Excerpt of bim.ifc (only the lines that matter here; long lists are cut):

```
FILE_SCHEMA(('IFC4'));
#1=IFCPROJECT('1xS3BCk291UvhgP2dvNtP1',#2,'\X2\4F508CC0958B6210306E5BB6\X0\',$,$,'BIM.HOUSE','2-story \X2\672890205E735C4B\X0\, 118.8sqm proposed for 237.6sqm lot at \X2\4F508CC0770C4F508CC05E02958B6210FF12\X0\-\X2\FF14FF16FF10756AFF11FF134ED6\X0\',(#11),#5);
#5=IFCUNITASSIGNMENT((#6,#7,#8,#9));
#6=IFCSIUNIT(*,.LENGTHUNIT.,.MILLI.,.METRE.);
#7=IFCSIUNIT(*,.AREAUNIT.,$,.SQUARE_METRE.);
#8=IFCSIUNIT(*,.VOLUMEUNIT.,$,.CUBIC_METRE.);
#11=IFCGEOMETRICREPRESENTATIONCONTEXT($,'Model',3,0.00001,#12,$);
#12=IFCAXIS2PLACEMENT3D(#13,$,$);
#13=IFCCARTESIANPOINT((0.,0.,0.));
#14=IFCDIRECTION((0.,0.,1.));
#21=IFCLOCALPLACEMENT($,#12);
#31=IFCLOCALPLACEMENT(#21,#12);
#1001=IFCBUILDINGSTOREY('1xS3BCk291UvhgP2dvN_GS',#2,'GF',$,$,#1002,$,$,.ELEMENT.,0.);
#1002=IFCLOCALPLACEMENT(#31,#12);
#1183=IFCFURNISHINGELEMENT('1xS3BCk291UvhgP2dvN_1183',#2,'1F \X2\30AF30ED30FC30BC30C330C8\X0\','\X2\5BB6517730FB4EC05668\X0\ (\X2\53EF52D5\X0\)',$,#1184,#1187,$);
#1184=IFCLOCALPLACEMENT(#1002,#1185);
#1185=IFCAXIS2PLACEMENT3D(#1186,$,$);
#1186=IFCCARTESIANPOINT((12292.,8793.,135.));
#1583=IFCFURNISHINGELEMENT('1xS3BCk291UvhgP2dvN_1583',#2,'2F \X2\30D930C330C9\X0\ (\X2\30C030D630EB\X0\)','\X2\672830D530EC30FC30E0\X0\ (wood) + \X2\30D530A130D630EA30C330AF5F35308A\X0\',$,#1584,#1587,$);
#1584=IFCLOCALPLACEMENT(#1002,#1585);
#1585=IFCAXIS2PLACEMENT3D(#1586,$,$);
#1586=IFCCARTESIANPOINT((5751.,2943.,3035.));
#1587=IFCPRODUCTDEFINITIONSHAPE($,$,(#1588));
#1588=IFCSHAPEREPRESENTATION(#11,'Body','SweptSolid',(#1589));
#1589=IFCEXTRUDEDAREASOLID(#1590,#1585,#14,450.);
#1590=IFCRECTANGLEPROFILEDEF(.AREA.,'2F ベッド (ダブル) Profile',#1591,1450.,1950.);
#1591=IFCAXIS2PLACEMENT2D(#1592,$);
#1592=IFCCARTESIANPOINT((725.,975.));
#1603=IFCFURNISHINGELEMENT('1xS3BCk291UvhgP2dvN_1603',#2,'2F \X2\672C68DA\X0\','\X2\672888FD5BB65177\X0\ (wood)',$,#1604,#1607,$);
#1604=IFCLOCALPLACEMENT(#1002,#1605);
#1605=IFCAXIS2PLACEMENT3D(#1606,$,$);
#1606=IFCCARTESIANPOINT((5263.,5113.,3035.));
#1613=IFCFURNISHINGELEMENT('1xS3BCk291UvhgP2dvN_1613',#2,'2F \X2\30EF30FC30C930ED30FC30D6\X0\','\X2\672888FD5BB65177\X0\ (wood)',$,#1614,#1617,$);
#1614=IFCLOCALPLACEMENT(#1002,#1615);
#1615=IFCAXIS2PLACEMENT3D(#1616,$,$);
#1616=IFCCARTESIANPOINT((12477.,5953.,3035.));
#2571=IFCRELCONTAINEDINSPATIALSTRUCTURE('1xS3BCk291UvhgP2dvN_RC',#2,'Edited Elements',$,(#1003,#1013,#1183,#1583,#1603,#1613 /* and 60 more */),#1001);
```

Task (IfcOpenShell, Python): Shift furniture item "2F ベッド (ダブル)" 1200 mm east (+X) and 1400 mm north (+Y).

```python
import ifcopenshell
import ifcopenshell.api.geometry
import ifcopenshell.util.placement

model = ifcopenshell.open("bim.ifc")

item = model.by_guid("1xS3BCk291UvhgP2dvN_1583")
matrix = ifcopenshell.util.placement.get_local_placement(item.ObjectPlacement)
matrix[0, 3] += 1200.0
matrix[1, 3] += 1400.0
ifcopenshell.api.geometry.edit_object_placement(model, product=item, matrix=matrix, is_si=False)

print(ifcopenshell.util.placement.get_local_placement(item.ObjectPlacement).round(3) + 0.0)

model.write("bim_edited.ifc")
```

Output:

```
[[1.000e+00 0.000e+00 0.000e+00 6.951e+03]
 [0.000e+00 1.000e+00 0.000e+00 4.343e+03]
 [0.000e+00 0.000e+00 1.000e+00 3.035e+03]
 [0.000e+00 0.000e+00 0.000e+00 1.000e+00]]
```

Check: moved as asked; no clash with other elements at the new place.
